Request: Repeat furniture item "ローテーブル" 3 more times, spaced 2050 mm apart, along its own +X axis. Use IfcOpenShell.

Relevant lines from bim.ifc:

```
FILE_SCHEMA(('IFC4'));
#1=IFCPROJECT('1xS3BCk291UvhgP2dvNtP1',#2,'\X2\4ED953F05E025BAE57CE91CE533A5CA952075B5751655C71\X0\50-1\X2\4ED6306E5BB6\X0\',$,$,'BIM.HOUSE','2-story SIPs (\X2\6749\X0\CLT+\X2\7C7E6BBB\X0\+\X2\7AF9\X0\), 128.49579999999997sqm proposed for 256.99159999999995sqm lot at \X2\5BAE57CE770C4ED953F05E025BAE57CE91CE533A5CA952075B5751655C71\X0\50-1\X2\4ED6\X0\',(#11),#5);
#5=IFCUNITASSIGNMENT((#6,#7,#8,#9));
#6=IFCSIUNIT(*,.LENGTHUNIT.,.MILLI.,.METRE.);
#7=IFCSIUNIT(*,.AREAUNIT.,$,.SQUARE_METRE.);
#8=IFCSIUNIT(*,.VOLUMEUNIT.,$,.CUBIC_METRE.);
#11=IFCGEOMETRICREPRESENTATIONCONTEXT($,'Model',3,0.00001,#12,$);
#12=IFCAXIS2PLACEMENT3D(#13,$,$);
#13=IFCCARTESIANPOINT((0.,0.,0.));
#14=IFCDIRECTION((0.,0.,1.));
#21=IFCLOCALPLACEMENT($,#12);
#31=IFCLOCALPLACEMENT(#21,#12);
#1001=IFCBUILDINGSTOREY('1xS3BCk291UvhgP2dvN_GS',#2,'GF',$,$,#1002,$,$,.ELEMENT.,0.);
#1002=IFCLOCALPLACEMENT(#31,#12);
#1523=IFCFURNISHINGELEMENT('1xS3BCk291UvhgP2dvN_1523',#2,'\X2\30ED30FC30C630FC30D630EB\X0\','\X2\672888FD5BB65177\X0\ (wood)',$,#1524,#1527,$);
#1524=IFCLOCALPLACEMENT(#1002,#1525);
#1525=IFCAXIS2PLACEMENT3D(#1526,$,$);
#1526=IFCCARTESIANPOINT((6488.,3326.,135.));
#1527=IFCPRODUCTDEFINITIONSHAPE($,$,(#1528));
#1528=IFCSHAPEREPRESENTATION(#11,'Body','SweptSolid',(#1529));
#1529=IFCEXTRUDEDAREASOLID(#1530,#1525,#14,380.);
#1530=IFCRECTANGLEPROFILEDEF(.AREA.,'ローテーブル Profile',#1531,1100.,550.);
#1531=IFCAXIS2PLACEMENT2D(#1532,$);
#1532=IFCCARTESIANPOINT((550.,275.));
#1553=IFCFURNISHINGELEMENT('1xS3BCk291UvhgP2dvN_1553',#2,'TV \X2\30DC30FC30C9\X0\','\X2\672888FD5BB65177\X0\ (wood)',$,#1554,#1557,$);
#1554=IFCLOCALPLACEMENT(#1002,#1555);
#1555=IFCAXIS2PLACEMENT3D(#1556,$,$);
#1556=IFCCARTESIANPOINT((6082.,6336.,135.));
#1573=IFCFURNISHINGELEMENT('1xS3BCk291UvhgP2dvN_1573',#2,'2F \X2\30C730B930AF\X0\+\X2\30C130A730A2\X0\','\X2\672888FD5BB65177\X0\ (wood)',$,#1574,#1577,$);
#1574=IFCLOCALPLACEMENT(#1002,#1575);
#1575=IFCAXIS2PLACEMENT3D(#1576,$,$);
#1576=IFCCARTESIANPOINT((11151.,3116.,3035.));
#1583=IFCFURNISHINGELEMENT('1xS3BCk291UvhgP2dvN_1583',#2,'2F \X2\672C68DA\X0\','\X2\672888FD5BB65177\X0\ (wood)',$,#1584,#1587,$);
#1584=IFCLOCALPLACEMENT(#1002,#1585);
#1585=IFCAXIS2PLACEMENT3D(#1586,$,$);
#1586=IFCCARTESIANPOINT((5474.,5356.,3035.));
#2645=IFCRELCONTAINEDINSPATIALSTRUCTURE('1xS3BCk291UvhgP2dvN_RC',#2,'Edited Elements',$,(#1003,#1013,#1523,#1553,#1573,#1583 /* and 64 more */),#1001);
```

```python
import ifcopenshell
import ifcopenshell.api.geometry
import ifcopenshell.api.root
import ifcopenshell.util.element
import ifcopenshell.util.placement
import ifcopenshell.util.unit

model = ifcopenshell.open("bim.ifc")
unit_scale = ifcopenshell.util.unit.calculate_unit_scale(model)


def reuse_history(source, copy):
    """copy_class also copies each property set's owner history, people and application; keep the originals."""
    for rel in copy.IsDefinedBy:
        if rel.is_a("IfcRelDefinesByProperties") and (history := rel.RelatingPropertyDefinition.OwnerHistory):
            rel.RelatingPropertyDefinition.OwnerHistory = source.OwnerHistory
            ifcopenshell.util.element.remove_deep2(model, history)


source = model.by_guid("1xS3BCk291UvhgP2dvN_1523")
base = ifcopenshell.util.placement.get_local_placement(source.ObjectPlacement)
step = base[:3, 0] * 2.05 / unit_scale

for i in range(1, 4):
    copy = ifcopenshell.api.root.copy_class(model, product=source)
    copy.Representation = ifcopenshell.util.element.copy_deep(
        model, source.Representation, exclude=["IfcGeometricRepresentationContext", "IfcRepresentationMap"]
    )
    reuse_history(source, copy)
    matrix = base.copy()
    matrix[:3, 3] += i * step
    print("added at", matrix[:3, 3].round(3) + 0.0)
    ifcopenshell.api.geometry.edit_object_placement(model, product=copy, matrix=matrix, is_si=False)

model.write("bim_v2.ifc")
```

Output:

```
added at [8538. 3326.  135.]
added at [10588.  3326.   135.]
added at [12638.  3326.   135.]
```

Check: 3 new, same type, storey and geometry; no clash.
